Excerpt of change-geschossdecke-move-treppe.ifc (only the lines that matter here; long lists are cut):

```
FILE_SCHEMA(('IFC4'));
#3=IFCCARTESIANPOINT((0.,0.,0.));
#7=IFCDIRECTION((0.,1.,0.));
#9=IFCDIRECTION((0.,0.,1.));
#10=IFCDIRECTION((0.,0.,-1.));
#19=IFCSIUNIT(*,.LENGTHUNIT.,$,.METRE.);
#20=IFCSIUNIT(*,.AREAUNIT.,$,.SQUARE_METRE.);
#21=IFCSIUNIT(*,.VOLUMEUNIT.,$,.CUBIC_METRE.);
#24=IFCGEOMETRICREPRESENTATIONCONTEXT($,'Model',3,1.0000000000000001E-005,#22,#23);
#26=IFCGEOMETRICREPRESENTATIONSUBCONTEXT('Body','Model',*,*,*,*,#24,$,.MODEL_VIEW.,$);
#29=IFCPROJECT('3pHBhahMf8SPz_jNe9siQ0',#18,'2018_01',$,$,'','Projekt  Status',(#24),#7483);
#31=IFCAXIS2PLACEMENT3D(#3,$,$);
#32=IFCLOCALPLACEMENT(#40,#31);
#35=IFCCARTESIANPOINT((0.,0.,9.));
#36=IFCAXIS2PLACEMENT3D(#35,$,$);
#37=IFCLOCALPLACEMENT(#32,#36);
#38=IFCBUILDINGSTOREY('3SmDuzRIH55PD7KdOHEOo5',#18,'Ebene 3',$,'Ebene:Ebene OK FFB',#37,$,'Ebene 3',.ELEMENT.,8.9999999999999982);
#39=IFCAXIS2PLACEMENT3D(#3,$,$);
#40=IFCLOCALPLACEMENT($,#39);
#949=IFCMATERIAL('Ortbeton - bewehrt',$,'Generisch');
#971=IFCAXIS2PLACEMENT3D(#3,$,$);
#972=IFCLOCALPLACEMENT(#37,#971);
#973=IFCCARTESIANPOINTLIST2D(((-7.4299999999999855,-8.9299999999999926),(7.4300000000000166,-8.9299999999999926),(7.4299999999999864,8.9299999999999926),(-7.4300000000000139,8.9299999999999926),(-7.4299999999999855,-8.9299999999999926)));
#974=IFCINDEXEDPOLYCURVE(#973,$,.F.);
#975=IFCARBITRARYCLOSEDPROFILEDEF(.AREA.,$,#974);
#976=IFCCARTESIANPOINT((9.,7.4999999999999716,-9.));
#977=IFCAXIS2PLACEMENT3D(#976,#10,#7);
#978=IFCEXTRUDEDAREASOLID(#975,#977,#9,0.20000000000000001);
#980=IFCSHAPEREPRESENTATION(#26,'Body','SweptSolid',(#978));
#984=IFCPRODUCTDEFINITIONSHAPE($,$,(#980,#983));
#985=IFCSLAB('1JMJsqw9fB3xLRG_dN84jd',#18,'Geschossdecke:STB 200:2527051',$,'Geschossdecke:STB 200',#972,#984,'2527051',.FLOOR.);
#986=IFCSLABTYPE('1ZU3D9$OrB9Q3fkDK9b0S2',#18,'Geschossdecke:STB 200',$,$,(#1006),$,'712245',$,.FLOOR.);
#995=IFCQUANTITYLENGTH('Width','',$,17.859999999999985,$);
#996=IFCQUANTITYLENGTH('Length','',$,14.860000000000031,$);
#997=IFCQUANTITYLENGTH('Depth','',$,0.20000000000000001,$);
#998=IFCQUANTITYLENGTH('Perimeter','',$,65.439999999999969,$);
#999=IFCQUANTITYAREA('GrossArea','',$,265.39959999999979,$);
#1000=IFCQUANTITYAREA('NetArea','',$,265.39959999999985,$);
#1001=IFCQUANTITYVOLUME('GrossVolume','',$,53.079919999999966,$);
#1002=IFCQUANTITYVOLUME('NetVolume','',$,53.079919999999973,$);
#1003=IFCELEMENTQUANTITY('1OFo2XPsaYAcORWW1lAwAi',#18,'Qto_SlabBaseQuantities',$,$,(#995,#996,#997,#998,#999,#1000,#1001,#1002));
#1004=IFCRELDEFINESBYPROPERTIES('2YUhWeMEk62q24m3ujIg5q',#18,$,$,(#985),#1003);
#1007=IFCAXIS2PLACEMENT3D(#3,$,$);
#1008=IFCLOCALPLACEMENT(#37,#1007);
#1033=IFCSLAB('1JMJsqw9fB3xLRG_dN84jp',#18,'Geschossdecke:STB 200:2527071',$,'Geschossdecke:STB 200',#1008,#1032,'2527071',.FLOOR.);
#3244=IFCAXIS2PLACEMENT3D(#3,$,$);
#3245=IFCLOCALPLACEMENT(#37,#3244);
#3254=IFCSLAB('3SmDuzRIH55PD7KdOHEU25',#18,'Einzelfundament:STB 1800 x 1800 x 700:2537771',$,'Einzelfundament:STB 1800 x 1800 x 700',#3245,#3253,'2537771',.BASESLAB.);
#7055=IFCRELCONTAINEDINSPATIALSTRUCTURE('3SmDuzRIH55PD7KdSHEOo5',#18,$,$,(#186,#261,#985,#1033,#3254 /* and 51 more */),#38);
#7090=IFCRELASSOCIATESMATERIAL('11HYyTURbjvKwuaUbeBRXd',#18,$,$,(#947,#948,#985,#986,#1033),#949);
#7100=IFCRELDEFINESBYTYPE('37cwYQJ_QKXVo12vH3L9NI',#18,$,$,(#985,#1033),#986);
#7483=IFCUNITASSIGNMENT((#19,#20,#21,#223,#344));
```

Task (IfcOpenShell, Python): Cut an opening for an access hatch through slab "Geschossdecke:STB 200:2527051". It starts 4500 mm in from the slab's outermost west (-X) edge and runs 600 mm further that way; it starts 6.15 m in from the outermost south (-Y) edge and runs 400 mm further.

```python
import numpy as np
import ifcopenshell
import ifcopenshell.api.feature
import ifcopenshell.api.geometry
import ifcopenshell.api.pset
import ifcopenshell.api.root
import ifcopenshell.geom
import ifcopenshell.util.element
import ifcopenshell.util.placement
import ifcopenshell.util.representation
import ifcopenshell.util.shape
import ifcopenshell.util.unit

model = ifcopenshell.open("change-geschossdecke-move-treppe.ifc")
unit_scale = ifcopenshell.util.unit.calculate_unit_scale(model)
area_scale = ifcopenshell.util.unit.calculate_unit_scale(model, "AREAUNIT")
volume_scale = ifcopenshell.util.unit.calculate_unit_scale(model, "VOLUMEUNIT")
settings = ifcopenshell.geom.settings()


def volume(element):
    """Net volume in cubic metres, openings subtracted."""
    shape = ifcopenshell.geom.create_shape(settings, element)
    return ifcopenshell.util.shape.get_volume(shape.geometry)


slab = model.by_id(985)
before = volume(slab)

# Extent in the slab's own axes, in metres. The edges named are its -X and -Y sides.
slab_shape = ifcopenshell.geom.create_shape(settings, slab)
vertices = ifcopenshell.util.shape.get_vertices(slab_shape.geometry)
x_min, y_min, bottom = vertices.min(axis=0)
top = vertices[:, 2].max()

opening = ifcopenshell.api.root.create_entity(model, ifc_class="IfcOpeningElement", name="Access hatch opening", predefined_type="OPENING")
context = ifcopenshell.util.representation.get_context(model, "Model", "Body", "MODEL_VIEW")
width, depth = 0.6, 0.4
outline = [(0.0, 0.0), (width, 0.0), (width, depth), (0.0, depth), (0.0, 0.0)]
# Overshoot both faces by 50 mm so the cut is clean.
shape = ifcopenshell.api.geometry.add_slab_representation(
    model, context=context, depth=top - bottom + 0.1, polyline=outline
)
ifcopenshell.api.geometry.assign_representation(model, product=opening, representation=shape)

matrix = ifcopenshell.util.placement.get_local_placement(slab.ObjectPlacement)
matrix[:, 3] = matrix @ np.append(np.array([x_min + 4.5, y_min + 6.15, bottom - 0.05]) / unit_scale, 1.0)
ifcopenshell.api.geometry.edit_object_placement(model, product=opening, matrix=matrix, is_si=False)
ifcopenshell.api.feature.add_feature(model, feature=opening, element=slab)

after = volume(slab)

# Update the slab's stored quantities.
qto = model.by_id(ifcopenshell.util.element.get_pset(slab, "Qto_SlabBaseQuantities", should_inherit=False)["id"])
ifcopenshell.api.pset.edit_qto(model, qto=qto, properties={
    "NetArea": after / (top - bottom) / area_scale,
    "NetVolume": after / volume_scale,
})

print(f"slab volume {before:.3f} -> {after:.3f} m3")

model.write("change-geschossdecke-move-treppe_v2.ifc")
```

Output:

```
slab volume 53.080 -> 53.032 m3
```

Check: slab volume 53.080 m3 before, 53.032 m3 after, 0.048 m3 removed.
